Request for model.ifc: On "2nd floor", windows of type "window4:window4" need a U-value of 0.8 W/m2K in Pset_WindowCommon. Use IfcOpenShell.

First a look at what the model holds.

```python
import ifcopenshell
import ifcopenshell.util.element

model = ifcopenshell.open("model.ifc")
print(model.schema)
storey = next(s for s in model.by_type("IfcBuildingStorey") if s.Name == "2nd floor")
windows = [e for e in ifcopenshell.util.element.get_decomposition(storey) if e.is_a("IfcWindow")]
seen = {}
for e in windows:
    element_type = ifcopenshell.util.element.get_type(e)
    key = (element_type.Name if element_type != e and element_type else None, ifcopenshell.util.element.get_pset(e, "Pset_WindowCommon", "ThermalTransmittance"))
    seen[key] = seen.get(key, 0) + 1
for (name, value), count in sorted(seen.items(), key=str):
    print(count, "x", name, "|", value)
```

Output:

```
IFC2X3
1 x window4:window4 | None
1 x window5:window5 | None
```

```python
import ifcopenshell
import ifcopenshell.api.pset
import ifcopenshell.util.element

model = ifcopenshell.open("model.ifc")

storey = next(s for s in model.by_type("IfcBuildingStorey") if s.Name == "2nd floor")
windows = [e for e in ifcopenshell.util.element.get_decomposition(storey) if e.is_a("IfcWindow")]

count = 0
for e in windows:
    element_type = ifcopenshell.util.element.get_type(e)
    if element_type in (None, e) or element_type.Name != "window4:window4":
        continue
    # add_pset returns the element's existing set when there is one.
    pset = ifcopenshell.api.pset.add_pset(model, product=e, name="Pset_WindowCommon")
    ifcopenshell.api.pset.edit_pset(model, pset=pset, properties={"ThermalTransmittance": 0.8})
    count += 1

print(count, "windows updated")

model.write("model_edited.ifc")
```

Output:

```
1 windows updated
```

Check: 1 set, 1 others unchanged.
